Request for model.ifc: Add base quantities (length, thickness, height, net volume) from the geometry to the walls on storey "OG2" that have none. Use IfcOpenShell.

First a look at what the model holds.

```python
import ifcopenshell
import ifcopenshell.util.element
import ifcopenshell.util.unit

model = ifcopenshell.open("model.ifc")
print(model.schema)
for unit_type in ("LENGTHUNIT", "AREAUNIT", "VOLUMEUNIT"):
    print(unit_type, ifcopenshell.util.unit.calculate_unit_scale(model, unit_type))
storey = next(s for s in model.by_type("IfcBuildingStorey") if s.Name == "OG2")
walls = [e for e in ifcopenshell.util.element.get_decomposition(storey) if e.is_a("IfcWall")]
for e in sorted(walls, key=lambda e: e.id()):
    print(e.id(), e.is_a(), e.Name, list(ifcopenshell.util.element.get_psets(e, qtos_only=True)), sep=" | ")
```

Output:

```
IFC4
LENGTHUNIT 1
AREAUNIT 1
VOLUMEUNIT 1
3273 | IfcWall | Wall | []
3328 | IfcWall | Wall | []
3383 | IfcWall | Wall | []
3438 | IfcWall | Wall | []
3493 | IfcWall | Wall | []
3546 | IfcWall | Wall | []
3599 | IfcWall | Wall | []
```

```python
import ifcopenshell
import ifcopenshell.api.pset
import ifcopenshell.geom
import ifcopenshell.util.element
import ifcopenshell.util.shape
import ifcopenshell.util.unit

model = ifcopenshell.open("model.ifc")
unit_scale = ifcopenshell.util.unit.calculate_unit_scale(model)
volume_scale = ifcopenshell.util.unit.calculate_unit_scale(model, "VOLUMEUNIT")
settings = ifcopenshell.geom.settings()

storey = next(s for s in model.by_type("IfcBuildingStorey") if s.Name == "OG2")
walls = [e for e in ifcopenshell.util.element.get_decomposition(storey) if e.is_a("IfcWall")]

for e in sorted(walls, key=lambda e: e.id()):
    if ifcopenshell.util.element.get_psets(e, qtos_only=True, should_inherit=False):
        continue
    # Geometry comes back in metres, in the element's own axes.
    shape = ifcopenshell.geom.create_shape(settings, e)
    values = {
        "Length": ifcopenshell.util.shape.get_x(shape.geometry) / unit_scale,
        "Width": ifcopenshell.util.shape.get_y(shape.geometry) / unit_scale,
        "Height": ifcopenshell.util.shape.get_z(shape.geometry) / unit_scale,
        "NetVolume": ifcopenshell.util.shape.get_volume(shape.geometry) / volume_scale,
    }
    qto = ifcopenshell.api.pset.add_qto(model, product=e, name="Qto_WallBaseQuantities")
    ifcopenshell.api.pset.edit_qto(model, qto=qto, properties=values)
    print(e.id(), {k: round(v, 3) for k, v in values.items()})

model.write("model_rev.ifc")
```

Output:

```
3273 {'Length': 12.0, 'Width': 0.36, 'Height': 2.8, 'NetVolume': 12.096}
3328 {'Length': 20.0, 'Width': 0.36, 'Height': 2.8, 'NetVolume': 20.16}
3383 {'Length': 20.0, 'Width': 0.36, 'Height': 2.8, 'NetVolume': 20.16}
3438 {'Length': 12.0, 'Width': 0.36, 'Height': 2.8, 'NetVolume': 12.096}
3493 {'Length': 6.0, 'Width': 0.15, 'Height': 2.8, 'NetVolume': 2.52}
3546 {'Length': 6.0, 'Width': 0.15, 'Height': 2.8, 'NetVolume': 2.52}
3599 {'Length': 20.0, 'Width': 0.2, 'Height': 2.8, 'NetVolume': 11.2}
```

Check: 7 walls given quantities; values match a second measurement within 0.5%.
